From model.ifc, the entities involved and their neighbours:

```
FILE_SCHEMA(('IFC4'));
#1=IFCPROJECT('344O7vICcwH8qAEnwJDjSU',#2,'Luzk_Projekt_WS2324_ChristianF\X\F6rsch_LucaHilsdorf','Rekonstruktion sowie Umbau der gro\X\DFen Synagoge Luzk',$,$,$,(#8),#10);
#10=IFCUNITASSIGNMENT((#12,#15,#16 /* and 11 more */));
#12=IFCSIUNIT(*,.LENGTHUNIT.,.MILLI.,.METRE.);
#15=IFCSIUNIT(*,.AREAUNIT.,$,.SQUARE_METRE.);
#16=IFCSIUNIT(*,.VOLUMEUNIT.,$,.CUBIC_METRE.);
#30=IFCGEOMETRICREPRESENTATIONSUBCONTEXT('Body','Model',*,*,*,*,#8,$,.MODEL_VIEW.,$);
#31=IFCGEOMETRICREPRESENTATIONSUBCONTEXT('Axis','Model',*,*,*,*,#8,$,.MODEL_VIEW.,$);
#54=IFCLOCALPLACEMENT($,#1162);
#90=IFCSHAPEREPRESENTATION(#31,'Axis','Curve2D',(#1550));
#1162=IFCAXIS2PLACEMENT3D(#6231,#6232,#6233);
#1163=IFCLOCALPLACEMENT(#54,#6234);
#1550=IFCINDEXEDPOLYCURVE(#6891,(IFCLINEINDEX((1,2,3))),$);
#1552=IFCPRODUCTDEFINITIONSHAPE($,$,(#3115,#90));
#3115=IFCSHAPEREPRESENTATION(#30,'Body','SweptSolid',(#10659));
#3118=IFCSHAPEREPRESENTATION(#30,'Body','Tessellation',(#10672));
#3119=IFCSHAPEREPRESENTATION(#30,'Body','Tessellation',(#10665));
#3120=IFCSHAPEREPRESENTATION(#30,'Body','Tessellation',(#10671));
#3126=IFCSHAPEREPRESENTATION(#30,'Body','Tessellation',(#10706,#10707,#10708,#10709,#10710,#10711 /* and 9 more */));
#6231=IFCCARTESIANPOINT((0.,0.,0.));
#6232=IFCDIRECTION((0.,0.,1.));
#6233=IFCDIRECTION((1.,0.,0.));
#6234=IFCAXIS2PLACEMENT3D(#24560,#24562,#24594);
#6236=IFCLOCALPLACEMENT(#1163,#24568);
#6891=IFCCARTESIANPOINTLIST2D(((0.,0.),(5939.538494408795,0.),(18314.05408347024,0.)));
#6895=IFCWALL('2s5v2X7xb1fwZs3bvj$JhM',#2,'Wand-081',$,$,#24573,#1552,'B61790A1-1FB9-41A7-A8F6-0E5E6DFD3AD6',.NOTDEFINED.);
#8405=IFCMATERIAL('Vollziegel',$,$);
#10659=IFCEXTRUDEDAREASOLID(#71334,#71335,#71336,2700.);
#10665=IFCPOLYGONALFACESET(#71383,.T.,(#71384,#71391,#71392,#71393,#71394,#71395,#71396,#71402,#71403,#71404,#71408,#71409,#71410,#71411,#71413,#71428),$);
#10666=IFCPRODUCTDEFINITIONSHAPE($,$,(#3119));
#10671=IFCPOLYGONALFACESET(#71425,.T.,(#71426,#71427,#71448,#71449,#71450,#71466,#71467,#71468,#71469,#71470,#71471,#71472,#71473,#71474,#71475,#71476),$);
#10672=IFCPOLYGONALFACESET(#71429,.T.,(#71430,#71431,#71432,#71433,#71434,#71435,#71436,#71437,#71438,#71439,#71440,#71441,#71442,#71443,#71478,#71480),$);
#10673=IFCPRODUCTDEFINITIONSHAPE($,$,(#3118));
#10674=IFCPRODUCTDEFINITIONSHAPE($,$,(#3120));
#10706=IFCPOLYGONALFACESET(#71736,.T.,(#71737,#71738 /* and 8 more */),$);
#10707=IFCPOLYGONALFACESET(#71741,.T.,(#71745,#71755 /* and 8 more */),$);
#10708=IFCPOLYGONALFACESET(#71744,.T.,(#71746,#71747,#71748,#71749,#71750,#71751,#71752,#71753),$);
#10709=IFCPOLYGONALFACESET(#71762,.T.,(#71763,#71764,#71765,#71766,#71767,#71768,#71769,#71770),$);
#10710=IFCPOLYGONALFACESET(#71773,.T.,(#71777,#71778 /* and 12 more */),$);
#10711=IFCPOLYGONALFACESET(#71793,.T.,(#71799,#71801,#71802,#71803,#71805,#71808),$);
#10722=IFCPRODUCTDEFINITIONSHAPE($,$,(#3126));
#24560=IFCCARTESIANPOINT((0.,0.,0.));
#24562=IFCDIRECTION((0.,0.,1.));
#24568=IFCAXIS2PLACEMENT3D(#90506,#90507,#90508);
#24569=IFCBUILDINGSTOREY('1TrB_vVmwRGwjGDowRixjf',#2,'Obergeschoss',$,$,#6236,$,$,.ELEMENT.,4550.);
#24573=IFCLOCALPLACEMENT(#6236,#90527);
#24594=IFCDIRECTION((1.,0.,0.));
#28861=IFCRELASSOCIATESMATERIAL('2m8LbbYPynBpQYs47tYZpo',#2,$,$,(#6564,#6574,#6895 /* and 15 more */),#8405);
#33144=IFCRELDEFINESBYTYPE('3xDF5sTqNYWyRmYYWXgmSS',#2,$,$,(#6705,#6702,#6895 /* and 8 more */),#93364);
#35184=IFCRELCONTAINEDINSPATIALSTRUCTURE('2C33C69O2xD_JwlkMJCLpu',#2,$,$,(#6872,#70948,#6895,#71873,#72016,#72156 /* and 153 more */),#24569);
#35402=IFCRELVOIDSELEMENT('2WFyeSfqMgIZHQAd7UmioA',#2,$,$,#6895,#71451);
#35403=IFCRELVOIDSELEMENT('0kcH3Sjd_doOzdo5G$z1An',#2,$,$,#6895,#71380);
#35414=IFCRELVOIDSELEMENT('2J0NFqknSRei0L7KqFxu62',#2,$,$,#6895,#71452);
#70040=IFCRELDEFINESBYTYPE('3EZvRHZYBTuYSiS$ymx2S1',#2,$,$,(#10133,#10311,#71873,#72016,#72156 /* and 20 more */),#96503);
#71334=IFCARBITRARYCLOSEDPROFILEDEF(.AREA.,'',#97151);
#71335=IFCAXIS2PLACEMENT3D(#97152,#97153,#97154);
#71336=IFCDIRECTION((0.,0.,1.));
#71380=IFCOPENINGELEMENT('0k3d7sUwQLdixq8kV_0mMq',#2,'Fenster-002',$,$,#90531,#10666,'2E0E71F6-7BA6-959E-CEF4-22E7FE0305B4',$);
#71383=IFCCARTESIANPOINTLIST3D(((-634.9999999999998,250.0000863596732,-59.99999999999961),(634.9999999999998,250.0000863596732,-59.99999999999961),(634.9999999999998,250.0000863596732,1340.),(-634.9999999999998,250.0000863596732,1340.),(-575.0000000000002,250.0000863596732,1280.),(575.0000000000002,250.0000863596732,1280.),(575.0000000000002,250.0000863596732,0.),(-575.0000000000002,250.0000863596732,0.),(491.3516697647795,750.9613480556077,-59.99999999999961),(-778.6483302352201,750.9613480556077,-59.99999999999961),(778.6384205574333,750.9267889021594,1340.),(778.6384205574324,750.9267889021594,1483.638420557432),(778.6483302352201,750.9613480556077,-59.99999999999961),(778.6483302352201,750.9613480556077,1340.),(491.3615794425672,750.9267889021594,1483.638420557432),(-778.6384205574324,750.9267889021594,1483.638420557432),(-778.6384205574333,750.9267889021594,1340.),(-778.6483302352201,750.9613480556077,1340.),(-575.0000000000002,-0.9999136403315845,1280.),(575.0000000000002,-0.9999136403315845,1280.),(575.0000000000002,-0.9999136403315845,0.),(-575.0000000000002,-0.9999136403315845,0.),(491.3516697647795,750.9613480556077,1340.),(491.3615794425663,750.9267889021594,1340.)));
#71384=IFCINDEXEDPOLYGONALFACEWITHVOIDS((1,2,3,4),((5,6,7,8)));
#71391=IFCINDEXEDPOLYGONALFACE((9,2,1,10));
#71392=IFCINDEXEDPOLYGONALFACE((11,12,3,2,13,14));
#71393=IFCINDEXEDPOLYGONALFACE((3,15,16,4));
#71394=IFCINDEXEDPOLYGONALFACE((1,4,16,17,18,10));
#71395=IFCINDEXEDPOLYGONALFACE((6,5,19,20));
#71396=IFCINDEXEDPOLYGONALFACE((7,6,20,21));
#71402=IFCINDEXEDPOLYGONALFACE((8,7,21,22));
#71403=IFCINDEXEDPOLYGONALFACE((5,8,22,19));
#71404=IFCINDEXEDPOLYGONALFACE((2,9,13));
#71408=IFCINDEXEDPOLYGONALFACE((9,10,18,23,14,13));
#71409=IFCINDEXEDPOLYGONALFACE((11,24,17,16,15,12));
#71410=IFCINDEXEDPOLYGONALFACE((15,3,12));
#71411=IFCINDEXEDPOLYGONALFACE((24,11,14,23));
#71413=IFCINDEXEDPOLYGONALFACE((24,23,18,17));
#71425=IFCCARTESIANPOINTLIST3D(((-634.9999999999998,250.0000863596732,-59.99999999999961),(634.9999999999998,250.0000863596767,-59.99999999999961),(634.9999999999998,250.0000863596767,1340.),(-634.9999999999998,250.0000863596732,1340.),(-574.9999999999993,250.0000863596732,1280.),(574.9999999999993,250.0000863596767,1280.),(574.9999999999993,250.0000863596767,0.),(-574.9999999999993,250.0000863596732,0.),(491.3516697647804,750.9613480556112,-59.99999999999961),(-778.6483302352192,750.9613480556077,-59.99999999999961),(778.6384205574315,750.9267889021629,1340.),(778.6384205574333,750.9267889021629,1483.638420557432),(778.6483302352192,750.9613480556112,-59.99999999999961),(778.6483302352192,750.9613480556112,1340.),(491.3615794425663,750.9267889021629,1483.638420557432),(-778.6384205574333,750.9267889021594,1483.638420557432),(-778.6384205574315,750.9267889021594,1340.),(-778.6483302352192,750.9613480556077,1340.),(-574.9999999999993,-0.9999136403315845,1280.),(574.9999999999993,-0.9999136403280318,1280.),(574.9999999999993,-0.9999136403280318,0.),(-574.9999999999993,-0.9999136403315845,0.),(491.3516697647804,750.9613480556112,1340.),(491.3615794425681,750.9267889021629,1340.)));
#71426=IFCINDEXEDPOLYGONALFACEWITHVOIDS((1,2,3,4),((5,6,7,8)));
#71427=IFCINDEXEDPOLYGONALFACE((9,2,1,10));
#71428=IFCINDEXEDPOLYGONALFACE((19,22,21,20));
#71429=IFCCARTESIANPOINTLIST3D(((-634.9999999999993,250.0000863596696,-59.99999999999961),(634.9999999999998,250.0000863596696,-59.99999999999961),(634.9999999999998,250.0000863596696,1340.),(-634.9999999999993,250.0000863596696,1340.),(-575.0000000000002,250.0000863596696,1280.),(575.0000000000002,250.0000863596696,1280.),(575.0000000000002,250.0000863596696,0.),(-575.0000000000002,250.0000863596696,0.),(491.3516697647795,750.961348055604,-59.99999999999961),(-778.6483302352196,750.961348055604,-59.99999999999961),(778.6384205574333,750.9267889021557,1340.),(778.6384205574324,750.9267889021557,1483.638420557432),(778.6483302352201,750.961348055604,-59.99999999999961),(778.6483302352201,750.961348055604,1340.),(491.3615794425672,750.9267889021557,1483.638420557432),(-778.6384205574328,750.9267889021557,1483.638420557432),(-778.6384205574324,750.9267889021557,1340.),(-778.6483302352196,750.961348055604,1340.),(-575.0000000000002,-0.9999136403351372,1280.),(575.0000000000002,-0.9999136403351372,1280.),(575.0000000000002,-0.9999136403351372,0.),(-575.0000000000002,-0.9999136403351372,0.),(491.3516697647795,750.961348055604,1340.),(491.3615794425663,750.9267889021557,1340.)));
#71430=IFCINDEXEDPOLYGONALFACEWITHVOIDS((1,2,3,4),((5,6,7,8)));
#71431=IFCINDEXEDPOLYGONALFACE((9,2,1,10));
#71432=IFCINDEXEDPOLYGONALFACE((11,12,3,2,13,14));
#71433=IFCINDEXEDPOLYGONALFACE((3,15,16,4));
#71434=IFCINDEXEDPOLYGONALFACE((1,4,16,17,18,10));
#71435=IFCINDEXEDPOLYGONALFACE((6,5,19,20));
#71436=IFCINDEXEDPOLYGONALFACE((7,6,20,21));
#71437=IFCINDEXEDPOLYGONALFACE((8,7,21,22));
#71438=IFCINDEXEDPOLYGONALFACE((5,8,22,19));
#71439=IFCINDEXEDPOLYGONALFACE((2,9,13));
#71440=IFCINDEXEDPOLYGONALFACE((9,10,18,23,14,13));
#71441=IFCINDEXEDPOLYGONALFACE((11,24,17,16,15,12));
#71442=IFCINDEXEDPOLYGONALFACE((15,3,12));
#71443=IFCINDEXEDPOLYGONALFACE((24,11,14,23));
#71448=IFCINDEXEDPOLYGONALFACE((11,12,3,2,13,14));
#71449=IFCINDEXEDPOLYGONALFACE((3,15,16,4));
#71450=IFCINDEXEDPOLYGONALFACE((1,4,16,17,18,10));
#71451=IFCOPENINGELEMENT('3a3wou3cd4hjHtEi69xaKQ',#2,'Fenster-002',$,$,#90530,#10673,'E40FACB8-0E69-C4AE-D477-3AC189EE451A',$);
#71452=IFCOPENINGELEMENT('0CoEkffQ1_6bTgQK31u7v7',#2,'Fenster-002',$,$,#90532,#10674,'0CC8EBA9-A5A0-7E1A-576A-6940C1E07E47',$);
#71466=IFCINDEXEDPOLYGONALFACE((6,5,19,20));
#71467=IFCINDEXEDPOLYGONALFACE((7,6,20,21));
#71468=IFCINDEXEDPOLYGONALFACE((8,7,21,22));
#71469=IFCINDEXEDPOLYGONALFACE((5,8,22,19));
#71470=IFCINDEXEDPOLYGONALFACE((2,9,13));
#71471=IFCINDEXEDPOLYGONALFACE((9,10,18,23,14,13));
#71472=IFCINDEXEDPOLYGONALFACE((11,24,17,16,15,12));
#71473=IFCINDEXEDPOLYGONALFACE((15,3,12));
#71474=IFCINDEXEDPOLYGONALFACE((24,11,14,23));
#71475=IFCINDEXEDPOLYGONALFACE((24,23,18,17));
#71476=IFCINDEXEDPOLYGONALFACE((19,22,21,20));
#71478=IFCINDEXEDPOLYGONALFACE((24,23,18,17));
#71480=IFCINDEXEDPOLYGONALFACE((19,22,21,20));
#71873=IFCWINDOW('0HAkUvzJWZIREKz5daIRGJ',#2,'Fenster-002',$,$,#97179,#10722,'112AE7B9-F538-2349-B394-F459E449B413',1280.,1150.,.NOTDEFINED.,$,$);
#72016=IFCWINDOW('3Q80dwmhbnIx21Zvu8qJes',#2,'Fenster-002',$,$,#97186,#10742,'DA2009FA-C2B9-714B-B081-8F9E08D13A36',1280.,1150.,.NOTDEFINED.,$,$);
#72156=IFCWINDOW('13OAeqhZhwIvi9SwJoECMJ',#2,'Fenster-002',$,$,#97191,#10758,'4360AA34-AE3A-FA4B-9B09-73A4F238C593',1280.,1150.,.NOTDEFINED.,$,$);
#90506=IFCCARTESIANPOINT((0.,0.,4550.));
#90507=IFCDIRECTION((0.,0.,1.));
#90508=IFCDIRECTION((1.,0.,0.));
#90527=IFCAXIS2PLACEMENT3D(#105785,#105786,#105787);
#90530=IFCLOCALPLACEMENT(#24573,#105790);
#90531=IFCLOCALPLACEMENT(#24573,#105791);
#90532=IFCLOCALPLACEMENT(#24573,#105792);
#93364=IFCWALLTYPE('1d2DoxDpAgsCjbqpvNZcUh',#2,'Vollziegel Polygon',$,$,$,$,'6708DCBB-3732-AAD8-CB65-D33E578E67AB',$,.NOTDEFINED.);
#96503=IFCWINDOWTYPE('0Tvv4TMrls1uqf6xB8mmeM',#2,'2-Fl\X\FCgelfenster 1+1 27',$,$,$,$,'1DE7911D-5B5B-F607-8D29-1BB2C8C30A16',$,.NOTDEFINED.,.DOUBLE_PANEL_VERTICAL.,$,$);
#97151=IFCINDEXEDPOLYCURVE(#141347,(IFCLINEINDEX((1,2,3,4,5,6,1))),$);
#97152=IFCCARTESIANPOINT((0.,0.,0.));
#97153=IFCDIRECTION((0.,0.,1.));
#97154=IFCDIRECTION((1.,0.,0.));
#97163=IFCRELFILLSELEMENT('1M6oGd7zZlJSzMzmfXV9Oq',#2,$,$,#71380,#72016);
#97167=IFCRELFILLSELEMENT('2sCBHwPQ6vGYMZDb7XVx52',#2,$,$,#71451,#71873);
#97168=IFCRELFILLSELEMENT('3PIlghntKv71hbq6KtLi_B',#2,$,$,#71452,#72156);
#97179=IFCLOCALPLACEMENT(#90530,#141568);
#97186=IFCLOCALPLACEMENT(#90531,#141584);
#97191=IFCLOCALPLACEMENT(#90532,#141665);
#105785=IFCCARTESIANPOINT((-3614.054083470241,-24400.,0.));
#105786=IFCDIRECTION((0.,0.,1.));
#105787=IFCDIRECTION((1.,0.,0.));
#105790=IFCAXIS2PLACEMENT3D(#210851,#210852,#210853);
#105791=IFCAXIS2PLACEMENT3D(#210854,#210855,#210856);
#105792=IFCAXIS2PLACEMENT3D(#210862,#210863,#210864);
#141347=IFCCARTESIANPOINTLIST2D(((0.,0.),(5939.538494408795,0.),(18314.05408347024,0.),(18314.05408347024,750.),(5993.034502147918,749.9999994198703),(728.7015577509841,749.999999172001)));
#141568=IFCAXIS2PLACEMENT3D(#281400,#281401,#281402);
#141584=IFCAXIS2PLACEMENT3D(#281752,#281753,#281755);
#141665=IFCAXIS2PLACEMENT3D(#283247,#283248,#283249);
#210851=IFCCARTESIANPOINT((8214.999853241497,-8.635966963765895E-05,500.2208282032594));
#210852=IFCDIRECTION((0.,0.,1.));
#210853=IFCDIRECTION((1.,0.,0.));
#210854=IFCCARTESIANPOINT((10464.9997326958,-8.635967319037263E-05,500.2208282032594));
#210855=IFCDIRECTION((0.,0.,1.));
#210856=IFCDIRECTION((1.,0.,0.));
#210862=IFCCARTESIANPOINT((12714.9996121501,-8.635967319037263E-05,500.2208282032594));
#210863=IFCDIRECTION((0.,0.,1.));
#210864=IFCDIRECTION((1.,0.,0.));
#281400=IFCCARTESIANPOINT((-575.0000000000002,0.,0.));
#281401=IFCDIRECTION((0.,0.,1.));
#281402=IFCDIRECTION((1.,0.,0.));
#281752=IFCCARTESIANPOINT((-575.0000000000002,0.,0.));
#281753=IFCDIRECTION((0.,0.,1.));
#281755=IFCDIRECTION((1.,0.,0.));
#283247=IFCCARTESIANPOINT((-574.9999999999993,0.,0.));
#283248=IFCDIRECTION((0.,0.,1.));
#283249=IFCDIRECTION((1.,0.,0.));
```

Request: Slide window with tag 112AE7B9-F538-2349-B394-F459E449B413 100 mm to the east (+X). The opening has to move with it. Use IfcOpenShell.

```python
import ifcopenshell
import ifcopenshell.api.geometry
import ifcopenshell.util.placement
import ifcopenshell.util.unit

model = ifcopenshell.open("model.ifc")
unit_scale = ifcopenshell.util.unit.calculate_unit_scale(model)

window = model.by_guid("0HAkUvzJWZIREKz5daIRGJ")
opening = window.FillsVoids[0].RelatingOpeningElement
wall = opening.VoidsElements[0].RelatingBuildingElement

wall_matrix = ifcopenshell.util.placement.get_local_placement(wall.ObjectPlacement)
shift = wall_matrix[:3, 0] * 0.1 / unit_scale
before = ifcopenshell.util.placement.get_local_placement(window.ObjectPlacement)[:3, 3].copy()

# The window is placed relative to its opening, so it follows when the opening moves.
matrix = ifcopenshell.util.placement.get_local_placement(opening.ObjectPlacement)
matrix[:3, 3] += shift
ifcopenshell.api.geometry.edit_object_placement(
    model, product=opening, matrix=matrix, is_si=False, should_transform_children=True
)

after = ifcopenshell.util.placement.get_local_placement(window.ObjectPlacement)[:3, 3]
print("window moved by", (after - before).round(3) + 0.0)

model.write("model_rev.ifc")
```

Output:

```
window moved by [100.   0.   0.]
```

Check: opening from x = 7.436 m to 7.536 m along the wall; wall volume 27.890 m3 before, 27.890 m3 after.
